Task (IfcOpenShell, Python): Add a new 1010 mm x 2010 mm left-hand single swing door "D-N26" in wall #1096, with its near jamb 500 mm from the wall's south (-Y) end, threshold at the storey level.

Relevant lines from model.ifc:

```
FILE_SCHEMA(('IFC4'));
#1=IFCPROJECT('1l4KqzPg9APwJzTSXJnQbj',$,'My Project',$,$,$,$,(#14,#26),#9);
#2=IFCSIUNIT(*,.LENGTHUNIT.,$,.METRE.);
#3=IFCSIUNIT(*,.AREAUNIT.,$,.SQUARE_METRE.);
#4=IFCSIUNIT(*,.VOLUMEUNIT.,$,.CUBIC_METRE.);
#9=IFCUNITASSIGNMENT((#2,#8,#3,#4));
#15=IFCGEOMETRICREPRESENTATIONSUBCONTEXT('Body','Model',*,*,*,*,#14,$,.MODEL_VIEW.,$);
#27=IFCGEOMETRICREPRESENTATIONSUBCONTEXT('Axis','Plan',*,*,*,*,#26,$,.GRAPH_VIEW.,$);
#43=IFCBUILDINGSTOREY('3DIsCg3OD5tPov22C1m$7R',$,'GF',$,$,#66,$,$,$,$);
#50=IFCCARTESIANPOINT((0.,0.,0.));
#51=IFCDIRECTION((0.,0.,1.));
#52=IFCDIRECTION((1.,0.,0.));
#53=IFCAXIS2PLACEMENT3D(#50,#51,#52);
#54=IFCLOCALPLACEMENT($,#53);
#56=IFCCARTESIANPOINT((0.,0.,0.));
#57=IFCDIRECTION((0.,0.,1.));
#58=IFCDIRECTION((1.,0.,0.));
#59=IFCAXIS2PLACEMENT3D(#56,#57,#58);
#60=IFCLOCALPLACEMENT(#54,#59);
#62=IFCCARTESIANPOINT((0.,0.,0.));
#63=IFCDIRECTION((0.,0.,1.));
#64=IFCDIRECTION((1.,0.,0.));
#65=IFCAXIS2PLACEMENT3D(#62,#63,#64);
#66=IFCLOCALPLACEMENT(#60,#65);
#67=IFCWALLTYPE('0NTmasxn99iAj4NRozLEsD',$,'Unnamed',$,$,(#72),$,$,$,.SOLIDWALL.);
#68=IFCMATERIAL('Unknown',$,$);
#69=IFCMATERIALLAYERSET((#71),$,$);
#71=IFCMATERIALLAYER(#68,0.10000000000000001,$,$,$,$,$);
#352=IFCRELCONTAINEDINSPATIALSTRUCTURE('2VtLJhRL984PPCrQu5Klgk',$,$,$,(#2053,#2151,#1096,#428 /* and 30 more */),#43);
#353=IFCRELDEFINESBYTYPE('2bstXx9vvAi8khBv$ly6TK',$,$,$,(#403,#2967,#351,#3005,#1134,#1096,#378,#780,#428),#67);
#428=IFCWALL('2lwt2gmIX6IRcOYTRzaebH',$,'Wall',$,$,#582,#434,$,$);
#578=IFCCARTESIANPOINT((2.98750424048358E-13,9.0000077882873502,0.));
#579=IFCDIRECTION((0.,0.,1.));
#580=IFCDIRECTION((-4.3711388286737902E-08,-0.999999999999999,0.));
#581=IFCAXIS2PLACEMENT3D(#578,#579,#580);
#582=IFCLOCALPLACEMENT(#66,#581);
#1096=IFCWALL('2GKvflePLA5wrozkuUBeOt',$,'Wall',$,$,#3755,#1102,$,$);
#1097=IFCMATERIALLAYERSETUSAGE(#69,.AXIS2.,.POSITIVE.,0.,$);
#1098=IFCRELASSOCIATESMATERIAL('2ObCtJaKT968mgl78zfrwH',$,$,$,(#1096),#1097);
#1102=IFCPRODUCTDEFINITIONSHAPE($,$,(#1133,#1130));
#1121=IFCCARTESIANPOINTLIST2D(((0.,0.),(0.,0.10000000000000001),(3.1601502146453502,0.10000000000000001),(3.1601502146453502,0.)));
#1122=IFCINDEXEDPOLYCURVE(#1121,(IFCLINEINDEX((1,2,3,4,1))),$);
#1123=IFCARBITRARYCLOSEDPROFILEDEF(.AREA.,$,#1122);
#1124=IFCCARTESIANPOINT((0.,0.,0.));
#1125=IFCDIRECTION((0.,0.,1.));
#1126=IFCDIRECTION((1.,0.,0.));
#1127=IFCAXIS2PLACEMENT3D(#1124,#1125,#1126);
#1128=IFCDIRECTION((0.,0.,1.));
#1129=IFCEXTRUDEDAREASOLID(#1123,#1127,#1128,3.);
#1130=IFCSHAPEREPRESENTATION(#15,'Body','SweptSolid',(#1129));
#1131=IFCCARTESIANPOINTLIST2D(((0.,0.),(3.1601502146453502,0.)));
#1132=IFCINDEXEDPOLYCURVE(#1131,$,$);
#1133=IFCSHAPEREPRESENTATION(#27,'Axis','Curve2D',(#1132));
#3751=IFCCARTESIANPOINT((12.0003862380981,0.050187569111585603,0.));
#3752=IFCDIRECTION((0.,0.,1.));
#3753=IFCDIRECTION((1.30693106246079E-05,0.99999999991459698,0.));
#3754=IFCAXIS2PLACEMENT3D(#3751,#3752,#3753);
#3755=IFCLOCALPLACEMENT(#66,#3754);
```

```python
import numpy as np
import ifcopenshell
import ifcopenshell.api.feature
import ifcopenshell.api.geometry
import ifcopenshell.api.root
import ifcopenshell.api.spatial
import ifcopenshell.geom
import ifcopenshell.util.element
import ifcopenshell.util.placement
import ifcopenshell.util.representation
import ifcopenshell.util.shape
import ifcopenshell.util.unit

model = ifcopenshell.open("model.ifc")
unit_scale = ifcopenshell.util.unit.calculate_unit_scale(model)
settings = ifcopenshell.geom.settings()


def volume(element):
    """Net volume in cubic metres, openings subtracted."""
    shape = ifcopenshell.geom.create_shape(settings, element)
    return ifcopenshell.util.shape.get_volume(shape.geometry)


wall = model.by_guid("2GKvflePLA5wrozkuUBeOt")
storey = ifcopenshell.util.element.get_container(wall, ifc_class="IfcBuildingStorey")
context = ifcopenshell.util.representation.get_context(model, "Model", "Body", "MODEL_VIEW")
before = volume(wall)

width, height, from_end, sill = 1.01, 2.01, 0.5, 0.0  # metres

# The wall runs along its own X axis, and the end named is its -X end.
wall_shape = ifcopenshell.geom.create_shape(settings, wall)
x, y, z = ifcopenshell.util.shape.get_vertices(wall_shape.geometry).T
start = x.min() + from_end
face, thickness = float(y.min()), float(y.max() - y.min())
wall_matrix = ifcopenshell.util.placement.get_local_placement(wall.ObjectPlacement)
level = ifcopenshell.util.placement.get_local_placement(storey.ObjectPlacement)[2, 3]


def in_wall(x, y):
    """Placement at x, y metres in the wall's axes, at sill height."""
    matrix = wall_matrix.copy()
    matrix[:, 3] = wall_matrix @ np.array([x / unit_scale, y / unit_scale, 0.0, 1.0])
    matrix[2, 3] = level + sill / unit_scale
    return matrix


# Opening: a box that overshoots both wall faces by 50 mm.
opening = ifcopenshell.api.root.create_entity(model, ifc_class="IfcOpeningElement", predefined_type="OPENING")
box = ifcopenshell.api.geometry.add_wall_representation(
    model, context=context, length=width, height=height, thickness=thickness + 0.1
)
ifcopenshell.api.geometry.assign_representation(model, product=opening, representation=box)
ifcopenshell.api.geometry.edit_object_placement(model, product=opening, matrix=in_wall(start, face - 0.05), is_si=False)
ifcopenshell.api.feature.add_feature(model, feature=opening, element=wall)

door = ifcopenshell.api.root.create_entity(model, ifc_class="IfcDoor", name="D-N26", predefined_type="DOOR")
door.OverallWidth, door.OverallHeight = width / unit_scale, height / unit_scale
door.OperationType = "SINGLE_SWING_LEFT"
body = ifcopenshell.api.geometry.add_door_representation(
    model,
    context=context,
    overall_width=door.OverallWidth,
    overall_height=door.OverallHeight,
    operation_type="SINGLE_SWING_LEFT",
    lining_properties={"LiningDepth": thickness / unit_scale, "ThresholdDepth": thickness / unit_scale},
)
ifcopenshell.api.geometry.assign_representation(model, product=door, representation=body)
ifcopenshell.api.spatial.assign_container(model, products=[door], relating_structure=storey)
ifcopenshell.api.feature.add_filling(model, opening=opening, element=door)

# The lining spans the wall, so the door starts at the wall face.
ifcopenshell.api.geometry.edit_object_placement(model, product=door, matrix=in_wall(start, face), is_si=False)

after = volume(wall)

print(f"wall volume {before:.3f} -> {after:.3f} m3")

model.write("model_rev.ifc")
```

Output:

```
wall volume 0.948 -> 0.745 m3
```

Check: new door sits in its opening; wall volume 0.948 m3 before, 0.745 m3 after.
